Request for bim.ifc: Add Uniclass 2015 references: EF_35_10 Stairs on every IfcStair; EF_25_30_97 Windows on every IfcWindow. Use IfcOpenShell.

First a look at what the model holds.

```python
import ifcopenshell

model = ifcopenshell.open("bim.ifc")
print(model.schema)
print("classifications:", [c.Name for c in model.by_type("IfcClassification")])
for ifc_class in ("IfcDoor", "IfcRoof", "IfcStair", "IfcWall", "IfcWindow"):
    print(ifc_class, len(model.by_type(ifc_class)))
```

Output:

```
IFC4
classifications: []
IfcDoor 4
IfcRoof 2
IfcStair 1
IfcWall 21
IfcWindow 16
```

```python
import ifcopenshell
import ifcopenshell.api.classification

model = ifcopenshell.open("bim.ifc")

system = ifcopenshell.api.classification.add_classification(model, classification="Uniclass 2015")

codes = {
    "IfcStair": ("EF_35_10", "Stairs"),
    "IfcWindow": ("EF_25_30_97", "Windows"),
}
for ifc_class, (code, name) in codes.items():
    products = model.by_type(ifc_class)
    ifcopenshell.api.classification.add_reference(
        model, products=products, classification=system, identification=code, name=name
    )
    print(code, len(products))

model.write("bim_updated.ifc")
```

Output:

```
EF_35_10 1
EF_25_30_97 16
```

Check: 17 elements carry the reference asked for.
